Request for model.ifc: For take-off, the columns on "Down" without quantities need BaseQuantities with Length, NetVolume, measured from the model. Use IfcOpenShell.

First a look at what the model holds.

```python
import ifcopenshell
import ifcopenshell.util.element
import ifcopenshell.util.unit

model = ifcopenshell.open("model.ifc")
print(model.schema)
for unit_type in ("LENGTHUNIT", "AREAUNIT", "VOLUMEUNIT"):
    print(unit_type, ifcopenshell.util.unit.calculate_unit_scale(model, unit_type))
storey = next(s for s in model.by_type("IfcBuildingStorey") if s.Name == "Down")
columns = [e for e in ifcopenshell.util.element.get_decomposition(storey) if e.is_a("IfcColumn")]
for e in sorted(columns, key=lambda e: e.id()):
    print(e.id(), e.is_a(), e.Name, list(ifcopenshell.util.element.get_psets(e, qtos_only=True)), sep=" | ")
```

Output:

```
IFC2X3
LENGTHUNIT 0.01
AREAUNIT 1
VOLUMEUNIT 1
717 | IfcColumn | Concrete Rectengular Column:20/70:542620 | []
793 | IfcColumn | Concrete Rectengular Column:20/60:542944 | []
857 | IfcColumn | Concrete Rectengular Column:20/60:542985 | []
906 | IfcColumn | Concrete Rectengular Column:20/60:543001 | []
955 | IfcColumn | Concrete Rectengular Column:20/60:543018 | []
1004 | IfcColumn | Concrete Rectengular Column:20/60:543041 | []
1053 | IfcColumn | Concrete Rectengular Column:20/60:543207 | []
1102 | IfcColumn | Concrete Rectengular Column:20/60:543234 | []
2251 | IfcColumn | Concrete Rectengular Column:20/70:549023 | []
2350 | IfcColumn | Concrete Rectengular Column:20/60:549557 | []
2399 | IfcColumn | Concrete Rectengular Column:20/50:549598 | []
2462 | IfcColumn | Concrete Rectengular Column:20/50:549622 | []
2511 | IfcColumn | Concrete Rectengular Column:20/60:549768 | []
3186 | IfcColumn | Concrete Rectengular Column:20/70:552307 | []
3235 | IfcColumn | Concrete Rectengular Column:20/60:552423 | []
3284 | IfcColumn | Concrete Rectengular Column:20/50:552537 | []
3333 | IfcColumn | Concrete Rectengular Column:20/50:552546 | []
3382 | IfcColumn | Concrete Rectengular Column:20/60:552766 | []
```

```python
import ifcopenshell
import ifcopenshell.api.pset
import ifcopenshell.geom
import ifcopenshell.util.element
import ifcopenshell.util.shape
import ifcopenshell.util.unit

model = ifcopenshell.open("model.ifc")
unit_scale = ifcopenshell.util.unit.calculate_unit_scale(model)
volume_scale = ifcopenshell.util.unit.calculate_unit_scale(model, "VOLUMEUNIT")
settings = ifcopenshell.geom.settings()

storey = next(s for s in model.by_type("IfcBuildingStorey") if s.Name == "Down")
columns = [e for e in ifcopenshell.util.element.get_decomposition(storey) if e.is_a("IfcColumn")]

for e in sorted(columns, key=lambda e: e.id()):
    if ifcopenshell.util.element.get_psets(e, qtos_only=True, should_inherit=False):
        continue
    # Geometry comes back in metres, in the element's own axes.
    shape = ifcopenshell.geom.create_shape(settings, e)
    values = {
        "Length": ifcopenshell.util.shape.get_z(shape.geometry) / unit_scale,
        "NetVolume": ifcopenshell.util.shape.get_volume(shape.geometry) / volume_scale,
    }
    qto = ifcopenshell.api.pset.add_qto(model, product=e, name="BaseQuantities")
    ifcopenshell.api.pset.edit_qto(model, qto=qto, properties=values)
    print(e.id(), {k: round(v, 3) for k, v in values.items()})

model.write("model_edited.ifc")
```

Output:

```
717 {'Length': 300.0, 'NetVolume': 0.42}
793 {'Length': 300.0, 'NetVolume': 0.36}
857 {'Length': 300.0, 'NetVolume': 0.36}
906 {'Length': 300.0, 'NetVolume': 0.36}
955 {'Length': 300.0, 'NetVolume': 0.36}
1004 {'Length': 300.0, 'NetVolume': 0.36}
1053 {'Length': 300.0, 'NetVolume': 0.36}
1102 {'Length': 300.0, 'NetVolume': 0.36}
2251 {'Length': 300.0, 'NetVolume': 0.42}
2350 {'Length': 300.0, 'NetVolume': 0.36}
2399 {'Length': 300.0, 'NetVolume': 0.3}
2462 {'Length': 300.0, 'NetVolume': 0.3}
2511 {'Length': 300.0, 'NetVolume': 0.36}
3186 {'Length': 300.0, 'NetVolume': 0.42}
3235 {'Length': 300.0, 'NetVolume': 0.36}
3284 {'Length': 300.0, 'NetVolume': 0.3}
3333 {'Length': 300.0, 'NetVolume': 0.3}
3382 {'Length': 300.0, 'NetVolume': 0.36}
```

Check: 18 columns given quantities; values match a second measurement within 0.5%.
